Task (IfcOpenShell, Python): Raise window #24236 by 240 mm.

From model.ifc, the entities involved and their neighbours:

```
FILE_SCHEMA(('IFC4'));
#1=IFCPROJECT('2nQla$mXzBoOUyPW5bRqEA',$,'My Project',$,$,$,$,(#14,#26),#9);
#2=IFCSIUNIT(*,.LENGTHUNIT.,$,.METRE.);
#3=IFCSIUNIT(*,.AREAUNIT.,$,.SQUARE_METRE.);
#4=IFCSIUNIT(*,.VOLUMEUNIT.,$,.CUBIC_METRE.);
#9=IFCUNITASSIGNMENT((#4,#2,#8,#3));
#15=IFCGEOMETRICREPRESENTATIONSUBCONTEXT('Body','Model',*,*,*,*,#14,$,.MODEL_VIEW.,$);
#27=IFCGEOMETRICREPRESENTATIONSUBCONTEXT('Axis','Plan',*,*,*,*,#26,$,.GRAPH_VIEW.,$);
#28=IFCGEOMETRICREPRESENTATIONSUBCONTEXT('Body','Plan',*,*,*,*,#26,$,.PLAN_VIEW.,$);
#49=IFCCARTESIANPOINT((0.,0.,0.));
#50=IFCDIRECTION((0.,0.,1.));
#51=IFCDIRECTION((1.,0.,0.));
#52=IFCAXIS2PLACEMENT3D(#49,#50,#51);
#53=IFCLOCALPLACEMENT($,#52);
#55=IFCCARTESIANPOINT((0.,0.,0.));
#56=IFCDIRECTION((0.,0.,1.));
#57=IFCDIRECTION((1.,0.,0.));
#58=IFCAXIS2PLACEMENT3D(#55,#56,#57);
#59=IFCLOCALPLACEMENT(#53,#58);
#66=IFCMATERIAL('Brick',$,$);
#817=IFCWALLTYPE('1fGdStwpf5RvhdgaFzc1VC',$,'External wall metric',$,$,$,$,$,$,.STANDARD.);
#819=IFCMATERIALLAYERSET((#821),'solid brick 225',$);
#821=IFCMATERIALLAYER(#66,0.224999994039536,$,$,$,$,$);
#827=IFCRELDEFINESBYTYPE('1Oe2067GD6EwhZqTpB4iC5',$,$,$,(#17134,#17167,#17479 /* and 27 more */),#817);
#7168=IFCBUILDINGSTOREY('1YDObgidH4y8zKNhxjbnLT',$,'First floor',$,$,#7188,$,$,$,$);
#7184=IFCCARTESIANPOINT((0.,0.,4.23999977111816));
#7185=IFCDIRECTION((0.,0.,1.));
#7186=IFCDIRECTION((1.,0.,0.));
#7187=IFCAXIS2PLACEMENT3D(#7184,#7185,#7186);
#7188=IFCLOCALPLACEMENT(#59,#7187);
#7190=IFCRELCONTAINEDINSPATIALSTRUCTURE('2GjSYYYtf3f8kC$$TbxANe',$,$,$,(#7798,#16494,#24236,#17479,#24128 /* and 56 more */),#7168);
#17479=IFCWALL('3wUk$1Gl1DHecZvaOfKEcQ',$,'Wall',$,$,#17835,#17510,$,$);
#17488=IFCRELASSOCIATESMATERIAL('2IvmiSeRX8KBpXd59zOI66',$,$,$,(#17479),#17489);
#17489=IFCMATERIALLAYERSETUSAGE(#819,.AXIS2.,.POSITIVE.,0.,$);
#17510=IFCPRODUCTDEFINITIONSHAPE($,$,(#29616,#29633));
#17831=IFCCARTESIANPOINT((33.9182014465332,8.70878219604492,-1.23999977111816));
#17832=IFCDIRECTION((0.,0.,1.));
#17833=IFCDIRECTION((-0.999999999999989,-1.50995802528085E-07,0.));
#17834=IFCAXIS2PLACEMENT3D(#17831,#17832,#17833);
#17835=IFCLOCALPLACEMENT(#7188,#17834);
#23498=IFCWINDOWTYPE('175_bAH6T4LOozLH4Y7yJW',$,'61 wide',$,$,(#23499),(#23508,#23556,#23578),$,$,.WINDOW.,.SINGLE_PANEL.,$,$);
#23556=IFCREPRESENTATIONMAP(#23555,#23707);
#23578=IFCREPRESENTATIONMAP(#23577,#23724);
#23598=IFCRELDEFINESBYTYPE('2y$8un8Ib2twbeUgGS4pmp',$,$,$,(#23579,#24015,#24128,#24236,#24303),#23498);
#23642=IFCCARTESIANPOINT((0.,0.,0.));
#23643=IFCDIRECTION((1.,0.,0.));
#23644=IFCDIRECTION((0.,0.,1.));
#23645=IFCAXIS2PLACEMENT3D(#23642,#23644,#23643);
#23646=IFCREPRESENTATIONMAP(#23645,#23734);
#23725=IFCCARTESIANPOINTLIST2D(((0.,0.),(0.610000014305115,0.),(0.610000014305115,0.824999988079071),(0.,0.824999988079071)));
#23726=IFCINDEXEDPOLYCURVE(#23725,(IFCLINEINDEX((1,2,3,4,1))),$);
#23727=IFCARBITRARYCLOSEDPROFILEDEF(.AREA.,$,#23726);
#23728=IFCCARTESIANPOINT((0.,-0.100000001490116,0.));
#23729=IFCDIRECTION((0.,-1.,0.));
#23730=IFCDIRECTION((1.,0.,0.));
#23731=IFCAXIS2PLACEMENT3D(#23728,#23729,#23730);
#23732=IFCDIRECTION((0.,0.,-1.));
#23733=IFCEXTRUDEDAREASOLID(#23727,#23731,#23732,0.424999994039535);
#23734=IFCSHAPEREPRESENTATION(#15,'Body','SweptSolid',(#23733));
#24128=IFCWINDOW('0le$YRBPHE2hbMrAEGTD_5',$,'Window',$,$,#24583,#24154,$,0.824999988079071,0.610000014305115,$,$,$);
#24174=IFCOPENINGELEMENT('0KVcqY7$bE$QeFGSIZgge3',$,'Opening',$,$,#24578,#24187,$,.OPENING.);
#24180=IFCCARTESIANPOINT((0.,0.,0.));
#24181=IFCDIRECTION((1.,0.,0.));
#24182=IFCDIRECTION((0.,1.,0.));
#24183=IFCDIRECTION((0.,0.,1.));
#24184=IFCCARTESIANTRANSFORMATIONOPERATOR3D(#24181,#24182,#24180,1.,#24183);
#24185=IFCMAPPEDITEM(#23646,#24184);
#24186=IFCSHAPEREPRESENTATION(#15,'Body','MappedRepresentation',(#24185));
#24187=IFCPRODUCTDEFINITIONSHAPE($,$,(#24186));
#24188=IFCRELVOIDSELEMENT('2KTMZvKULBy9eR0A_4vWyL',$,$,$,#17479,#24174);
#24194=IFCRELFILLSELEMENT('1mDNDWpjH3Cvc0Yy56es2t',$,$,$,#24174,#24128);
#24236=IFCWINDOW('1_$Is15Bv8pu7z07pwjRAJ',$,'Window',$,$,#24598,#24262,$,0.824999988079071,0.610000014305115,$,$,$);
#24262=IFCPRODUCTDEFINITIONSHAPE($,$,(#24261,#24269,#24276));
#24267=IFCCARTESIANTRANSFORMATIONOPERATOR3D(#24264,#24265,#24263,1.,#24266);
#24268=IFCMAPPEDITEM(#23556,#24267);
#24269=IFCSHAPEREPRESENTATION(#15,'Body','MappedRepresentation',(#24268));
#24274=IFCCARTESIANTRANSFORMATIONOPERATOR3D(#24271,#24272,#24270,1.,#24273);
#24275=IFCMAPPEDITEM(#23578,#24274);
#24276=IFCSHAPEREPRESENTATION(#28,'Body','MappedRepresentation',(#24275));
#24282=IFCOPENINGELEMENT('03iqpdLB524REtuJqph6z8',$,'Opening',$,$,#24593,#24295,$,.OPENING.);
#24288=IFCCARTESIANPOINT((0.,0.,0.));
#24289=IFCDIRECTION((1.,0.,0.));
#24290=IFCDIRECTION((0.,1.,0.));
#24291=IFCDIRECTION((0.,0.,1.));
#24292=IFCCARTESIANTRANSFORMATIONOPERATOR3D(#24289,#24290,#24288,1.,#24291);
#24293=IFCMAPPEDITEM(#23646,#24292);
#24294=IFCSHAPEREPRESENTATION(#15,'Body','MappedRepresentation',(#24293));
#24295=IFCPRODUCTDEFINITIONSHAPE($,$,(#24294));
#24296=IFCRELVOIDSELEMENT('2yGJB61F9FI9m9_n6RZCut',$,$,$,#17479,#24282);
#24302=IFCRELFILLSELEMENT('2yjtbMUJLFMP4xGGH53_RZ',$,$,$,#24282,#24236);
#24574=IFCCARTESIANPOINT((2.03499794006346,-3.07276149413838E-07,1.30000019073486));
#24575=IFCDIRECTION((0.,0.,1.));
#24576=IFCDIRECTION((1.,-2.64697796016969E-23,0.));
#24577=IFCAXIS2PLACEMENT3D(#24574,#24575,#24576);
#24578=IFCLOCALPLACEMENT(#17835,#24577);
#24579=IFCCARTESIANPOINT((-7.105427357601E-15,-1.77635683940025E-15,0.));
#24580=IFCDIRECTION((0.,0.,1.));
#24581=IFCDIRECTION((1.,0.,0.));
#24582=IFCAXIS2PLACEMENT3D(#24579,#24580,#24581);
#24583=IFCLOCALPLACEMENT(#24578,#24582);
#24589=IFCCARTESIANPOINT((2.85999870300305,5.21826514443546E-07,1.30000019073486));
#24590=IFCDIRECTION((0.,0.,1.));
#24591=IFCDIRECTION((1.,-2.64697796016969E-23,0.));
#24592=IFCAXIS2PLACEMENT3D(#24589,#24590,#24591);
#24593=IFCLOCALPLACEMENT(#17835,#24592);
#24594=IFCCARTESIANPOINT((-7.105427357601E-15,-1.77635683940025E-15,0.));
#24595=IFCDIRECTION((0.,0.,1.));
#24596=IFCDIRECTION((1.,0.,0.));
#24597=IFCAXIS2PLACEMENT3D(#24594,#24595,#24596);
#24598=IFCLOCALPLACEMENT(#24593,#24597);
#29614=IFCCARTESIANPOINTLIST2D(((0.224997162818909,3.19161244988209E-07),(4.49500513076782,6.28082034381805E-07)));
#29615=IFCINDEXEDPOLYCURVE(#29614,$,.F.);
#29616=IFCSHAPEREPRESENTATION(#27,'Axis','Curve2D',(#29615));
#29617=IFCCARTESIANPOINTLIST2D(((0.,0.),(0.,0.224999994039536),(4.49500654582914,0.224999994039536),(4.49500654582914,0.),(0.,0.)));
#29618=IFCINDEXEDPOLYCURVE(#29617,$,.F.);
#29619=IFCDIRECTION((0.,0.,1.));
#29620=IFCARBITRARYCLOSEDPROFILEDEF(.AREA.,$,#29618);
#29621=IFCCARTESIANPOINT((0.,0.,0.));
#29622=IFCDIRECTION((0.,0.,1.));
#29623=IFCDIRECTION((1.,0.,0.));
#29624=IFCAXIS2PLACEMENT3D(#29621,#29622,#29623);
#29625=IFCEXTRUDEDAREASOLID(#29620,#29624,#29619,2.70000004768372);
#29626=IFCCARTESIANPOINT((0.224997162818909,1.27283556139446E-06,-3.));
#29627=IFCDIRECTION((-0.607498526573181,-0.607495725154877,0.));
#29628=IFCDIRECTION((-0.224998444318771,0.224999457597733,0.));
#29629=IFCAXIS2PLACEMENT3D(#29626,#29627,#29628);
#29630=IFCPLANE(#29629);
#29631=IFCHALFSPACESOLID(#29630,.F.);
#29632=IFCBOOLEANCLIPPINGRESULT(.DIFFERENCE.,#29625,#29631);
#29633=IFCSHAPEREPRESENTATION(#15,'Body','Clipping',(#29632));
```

```python
import numpy as np
import ifcopenshell
import ifcopenshell.api.geometry
import ifcopenshell.util.placement
import ifcopenshell.util.unit

model = ifcopenshell.open("model.ifc")
unit_scale = ifcopenshell.util.unit.calculate_unit_scale(model)

window = model.by_guid("1_$Is15Bv8pu7z07pwjRAJ")
opening = window.FillsVoids[0].RelatingOpeningElement
dz = 0.24 / unit_scale

shift = np.array([0.0, 0.0, dz])
# The window is placed relative to its opening, so it follows when the opening moves.
matrix = ifcopenshell.util.placement.get_local_placement(opening.ObjectPlacement)
matrix[:3, 3] += shift
ifcopenshell.api.geometry.edit_object_placement(
    model, product=opening, matrix=matrix, is_si=False, should_transform_children=True
)

print(f"moved by {dz * unit_scale:+.3f} m")

model.write("model_updated.ifc")
```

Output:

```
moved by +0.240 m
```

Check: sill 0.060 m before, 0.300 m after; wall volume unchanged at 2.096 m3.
